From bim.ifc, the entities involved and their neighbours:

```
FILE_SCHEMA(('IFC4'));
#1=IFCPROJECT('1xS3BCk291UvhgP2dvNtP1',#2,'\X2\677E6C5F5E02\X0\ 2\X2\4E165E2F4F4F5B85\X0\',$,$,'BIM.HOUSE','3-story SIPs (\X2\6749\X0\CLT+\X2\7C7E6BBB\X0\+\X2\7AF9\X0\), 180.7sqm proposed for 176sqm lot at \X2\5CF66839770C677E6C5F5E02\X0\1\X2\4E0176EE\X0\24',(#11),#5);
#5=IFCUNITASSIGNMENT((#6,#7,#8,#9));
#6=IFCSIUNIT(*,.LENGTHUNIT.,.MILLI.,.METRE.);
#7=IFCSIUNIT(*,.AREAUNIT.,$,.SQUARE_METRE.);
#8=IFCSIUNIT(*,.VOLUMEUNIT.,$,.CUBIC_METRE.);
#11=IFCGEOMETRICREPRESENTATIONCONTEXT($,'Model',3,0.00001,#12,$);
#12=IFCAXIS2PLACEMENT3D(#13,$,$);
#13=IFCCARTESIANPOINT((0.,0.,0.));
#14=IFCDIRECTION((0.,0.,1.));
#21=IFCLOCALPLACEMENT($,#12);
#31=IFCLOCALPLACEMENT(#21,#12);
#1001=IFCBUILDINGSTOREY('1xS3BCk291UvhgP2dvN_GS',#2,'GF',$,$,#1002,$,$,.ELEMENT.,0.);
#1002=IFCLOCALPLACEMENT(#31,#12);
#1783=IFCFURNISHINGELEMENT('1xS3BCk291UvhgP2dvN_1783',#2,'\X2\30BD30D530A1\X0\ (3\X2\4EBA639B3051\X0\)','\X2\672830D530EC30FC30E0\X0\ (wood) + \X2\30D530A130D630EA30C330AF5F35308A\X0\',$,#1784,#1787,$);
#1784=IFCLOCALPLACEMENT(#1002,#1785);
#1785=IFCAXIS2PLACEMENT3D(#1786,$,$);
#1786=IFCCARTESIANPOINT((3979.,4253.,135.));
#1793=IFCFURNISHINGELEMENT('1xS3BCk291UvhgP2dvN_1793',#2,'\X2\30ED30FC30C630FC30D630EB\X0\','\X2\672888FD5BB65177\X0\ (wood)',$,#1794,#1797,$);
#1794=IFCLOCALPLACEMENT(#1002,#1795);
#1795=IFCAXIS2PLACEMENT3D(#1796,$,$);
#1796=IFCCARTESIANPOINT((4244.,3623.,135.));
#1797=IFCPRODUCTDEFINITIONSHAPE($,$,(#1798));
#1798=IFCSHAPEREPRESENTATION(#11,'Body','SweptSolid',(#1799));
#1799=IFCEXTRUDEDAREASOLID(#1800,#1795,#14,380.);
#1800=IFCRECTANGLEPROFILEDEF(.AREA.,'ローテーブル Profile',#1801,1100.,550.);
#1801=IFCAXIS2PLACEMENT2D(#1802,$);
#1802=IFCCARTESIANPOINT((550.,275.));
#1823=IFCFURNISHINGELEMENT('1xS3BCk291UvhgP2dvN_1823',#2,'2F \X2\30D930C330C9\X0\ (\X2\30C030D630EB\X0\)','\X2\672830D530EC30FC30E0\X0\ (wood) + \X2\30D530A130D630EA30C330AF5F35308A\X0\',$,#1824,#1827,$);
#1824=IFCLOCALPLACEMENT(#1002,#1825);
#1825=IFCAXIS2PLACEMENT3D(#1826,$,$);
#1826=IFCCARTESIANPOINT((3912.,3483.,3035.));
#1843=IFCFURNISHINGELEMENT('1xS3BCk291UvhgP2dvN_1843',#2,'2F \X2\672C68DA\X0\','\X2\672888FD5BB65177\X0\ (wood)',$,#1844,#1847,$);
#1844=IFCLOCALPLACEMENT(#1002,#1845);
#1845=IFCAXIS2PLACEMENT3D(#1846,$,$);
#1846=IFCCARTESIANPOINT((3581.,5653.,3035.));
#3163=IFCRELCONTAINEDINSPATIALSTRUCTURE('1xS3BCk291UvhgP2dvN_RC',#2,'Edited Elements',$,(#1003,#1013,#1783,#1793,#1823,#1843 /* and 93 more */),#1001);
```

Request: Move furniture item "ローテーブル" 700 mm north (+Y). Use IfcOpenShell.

```python
import ifcopenshell
import ifcopenshell.api.geometry
import ifcopenshell.util.placement
import ifcopenshell.util.unit

model = ifcopenshell.open("bim.ifc")
unit_scale = ifcopenshell.util.unit.calculate_unit_scale(model)

item = model.by_guid("1xS3BCk291UvhgP2dvN_1793")
matrix = ifcopenshell.util.placement.get_local_placement(item.ObjectPlacement)
matrix[1, 3] += 0.7 / unit_scale
ifcopenshell.api.geometry.edit_object_placement(model, product=item, matrix=matrix, is_si=False)

print(ifcopenshell.util.placement.get_local_placement(item.ObjectPlacement).round(3) + 0.0)

model.write("bim_rev.ifc")
```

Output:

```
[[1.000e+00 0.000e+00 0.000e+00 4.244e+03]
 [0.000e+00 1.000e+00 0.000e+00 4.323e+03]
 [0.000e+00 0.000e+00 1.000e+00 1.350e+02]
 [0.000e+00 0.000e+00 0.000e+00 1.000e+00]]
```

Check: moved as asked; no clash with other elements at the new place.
